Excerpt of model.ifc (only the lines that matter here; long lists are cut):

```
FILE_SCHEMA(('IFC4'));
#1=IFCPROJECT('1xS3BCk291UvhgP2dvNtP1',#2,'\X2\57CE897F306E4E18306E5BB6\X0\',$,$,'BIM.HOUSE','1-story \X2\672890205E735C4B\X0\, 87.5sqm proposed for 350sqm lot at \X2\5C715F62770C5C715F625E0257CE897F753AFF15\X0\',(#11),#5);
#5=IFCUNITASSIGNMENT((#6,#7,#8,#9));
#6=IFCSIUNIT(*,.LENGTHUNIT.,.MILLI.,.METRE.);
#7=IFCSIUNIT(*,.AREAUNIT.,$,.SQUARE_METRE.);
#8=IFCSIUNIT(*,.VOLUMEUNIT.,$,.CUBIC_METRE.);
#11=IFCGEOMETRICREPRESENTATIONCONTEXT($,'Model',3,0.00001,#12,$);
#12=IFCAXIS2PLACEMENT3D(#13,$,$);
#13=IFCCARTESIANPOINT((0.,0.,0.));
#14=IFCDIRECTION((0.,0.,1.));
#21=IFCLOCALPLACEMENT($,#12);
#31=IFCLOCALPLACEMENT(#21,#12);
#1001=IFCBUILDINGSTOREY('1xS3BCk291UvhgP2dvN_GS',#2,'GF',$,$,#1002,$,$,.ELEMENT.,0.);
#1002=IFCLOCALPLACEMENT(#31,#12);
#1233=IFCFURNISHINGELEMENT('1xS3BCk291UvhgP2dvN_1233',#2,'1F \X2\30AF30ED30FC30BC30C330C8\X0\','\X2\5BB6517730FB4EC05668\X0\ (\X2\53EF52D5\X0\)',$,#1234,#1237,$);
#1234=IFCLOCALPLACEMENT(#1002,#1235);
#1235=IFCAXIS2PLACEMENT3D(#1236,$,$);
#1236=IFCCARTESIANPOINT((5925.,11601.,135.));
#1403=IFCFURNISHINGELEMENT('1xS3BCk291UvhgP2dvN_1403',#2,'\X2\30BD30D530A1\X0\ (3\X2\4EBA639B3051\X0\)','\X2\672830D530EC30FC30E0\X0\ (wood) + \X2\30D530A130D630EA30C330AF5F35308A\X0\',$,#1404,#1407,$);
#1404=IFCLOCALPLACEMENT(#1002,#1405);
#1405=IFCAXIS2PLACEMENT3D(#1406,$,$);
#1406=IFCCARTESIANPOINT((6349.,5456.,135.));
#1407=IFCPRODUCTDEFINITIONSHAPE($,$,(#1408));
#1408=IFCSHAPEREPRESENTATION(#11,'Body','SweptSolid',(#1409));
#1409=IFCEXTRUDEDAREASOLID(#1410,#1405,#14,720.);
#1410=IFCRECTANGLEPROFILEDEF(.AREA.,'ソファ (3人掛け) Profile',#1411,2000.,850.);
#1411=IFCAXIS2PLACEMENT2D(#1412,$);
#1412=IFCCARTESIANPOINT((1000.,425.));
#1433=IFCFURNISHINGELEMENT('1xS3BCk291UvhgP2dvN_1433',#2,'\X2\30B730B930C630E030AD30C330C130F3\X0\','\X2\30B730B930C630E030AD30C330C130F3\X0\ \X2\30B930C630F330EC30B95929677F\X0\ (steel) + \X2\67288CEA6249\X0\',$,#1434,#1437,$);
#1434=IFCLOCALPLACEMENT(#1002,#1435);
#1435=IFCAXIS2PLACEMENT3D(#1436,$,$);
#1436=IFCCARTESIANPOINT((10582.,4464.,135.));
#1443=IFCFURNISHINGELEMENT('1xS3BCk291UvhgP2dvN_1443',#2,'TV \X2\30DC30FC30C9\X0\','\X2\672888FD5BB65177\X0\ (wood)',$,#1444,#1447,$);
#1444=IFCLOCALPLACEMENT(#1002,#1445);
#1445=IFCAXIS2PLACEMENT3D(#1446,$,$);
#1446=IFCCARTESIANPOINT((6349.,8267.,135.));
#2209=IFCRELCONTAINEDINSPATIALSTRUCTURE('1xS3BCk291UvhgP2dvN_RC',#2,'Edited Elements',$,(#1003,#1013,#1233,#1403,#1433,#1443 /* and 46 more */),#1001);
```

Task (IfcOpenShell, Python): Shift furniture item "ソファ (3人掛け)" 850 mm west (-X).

```python
import ifcopenshell
import ifcopenshell.api.geometry
import ifcopenshell.util.placement

model = ifcopenshell.open("model.ifc")

item = model.by_id(1403)
matrix = ifcopenshell.util.placement.get_local_placement(item.ObjectPlacement)
matrix[0, 3] -= 850.0
ifcopenshell.api.geometry.edit_object_placement(model, product=item, matrix=matrix, is_si=False)

print(ifcopenshell.util.placement.get_local_placement(item.ObjectPlacement).round(3) + 0.0)

model.write("model-out.ifc")
```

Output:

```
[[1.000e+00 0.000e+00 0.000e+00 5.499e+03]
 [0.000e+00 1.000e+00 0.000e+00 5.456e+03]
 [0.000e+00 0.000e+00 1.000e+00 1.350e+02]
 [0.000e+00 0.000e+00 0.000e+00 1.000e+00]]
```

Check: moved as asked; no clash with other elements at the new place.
